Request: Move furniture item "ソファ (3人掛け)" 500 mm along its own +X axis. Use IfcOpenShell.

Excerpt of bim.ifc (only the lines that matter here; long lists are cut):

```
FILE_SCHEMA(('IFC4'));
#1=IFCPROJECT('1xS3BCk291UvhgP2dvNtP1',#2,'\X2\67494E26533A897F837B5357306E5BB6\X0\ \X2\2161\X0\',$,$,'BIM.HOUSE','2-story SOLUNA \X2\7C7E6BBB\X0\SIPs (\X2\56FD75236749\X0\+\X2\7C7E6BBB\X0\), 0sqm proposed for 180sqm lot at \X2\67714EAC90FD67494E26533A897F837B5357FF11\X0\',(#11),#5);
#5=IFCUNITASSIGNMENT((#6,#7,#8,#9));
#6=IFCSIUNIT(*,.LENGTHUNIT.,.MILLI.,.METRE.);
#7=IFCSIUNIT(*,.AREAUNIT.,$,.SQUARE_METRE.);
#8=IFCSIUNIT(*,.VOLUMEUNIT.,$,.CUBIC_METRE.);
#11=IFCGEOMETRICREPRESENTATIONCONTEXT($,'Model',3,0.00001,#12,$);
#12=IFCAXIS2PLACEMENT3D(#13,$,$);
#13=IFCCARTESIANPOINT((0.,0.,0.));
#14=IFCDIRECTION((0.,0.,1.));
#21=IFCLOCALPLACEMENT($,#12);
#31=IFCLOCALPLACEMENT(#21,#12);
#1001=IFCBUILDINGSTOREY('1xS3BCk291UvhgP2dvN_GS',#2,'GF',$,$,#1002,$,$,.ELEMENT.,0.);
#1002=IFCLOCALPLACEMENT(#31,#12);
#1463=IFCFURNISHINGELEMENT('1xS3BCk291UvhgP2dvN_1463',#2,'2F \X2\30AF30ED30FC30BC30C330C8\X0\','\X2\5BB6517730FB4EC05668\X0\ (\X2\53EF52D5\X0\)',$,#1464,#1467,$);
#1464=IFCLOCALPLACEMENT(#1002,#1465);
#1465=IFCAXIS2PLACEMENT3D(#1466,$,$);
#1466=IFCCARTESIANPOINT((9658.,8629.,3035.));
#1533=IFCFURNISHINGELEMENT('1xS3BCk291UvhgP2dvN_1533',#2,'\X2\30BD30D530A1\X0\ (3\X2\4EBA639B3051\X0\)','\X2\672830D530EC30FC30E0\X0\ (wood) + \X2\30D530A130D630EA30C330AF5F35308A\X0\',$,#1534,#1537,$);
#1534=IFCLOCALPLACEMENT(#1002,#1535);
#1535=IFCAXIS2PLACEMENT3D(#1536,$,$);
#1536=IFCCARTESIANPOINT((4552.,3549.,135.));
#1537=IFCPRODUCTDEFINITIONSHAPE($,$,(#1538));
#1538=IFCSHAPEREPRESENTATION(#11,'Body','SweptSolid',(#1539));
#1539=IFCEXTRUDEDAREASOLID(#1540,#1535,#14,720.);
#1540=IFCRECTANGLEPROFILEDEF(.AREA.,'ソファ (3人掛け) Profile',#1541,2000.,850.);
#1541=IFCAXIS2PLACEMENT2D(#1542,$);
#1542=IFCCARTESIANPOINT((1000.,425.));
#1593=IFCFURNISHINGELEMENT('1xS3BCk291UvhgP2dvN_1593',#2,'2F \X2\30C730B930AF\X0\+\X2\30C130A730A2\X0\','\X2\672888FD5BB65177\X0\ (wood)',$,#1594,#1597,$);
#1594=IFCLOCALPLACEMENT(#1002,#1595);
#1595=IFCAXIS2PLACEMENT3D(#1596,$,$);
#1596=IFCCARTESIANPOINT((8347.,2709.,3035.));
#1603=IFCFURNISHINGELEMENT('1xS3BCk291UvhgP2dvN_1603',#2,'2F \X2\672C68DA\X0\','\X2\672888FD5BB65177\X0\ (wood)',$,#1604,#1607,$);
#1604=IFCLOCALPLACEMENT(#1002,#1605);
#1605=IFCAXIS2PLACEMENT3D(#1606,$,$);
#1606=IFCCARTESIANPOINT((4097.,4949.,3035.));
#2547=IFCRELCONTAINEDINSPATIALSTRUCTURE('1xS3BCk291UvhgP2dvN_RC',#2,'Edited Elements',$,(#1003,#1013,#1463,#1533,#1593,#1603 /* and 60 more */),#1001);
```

```python
import ifcopenshell
import ifcopenshell.api.geometry
import ifcopenshell.util.placement

model = ifcopenshell.open("bim.ifc")

item = model.by_id(1533)
matrix = ifcopenshell.util.placement.get_local_placement(item.ObjectPlacement)
matrix[:3, 3] += matrix[:3, 0] * 500.0
ifcopenshell.api.geometry.edit_object_placement(model, product=item, matrix=matrix, is_si=False)

print(ifcopenshell.util.placement.get_local_placement(item.ObjectPlacement).round(3) + 0.0)

model.write("bim_rev.ifc")
```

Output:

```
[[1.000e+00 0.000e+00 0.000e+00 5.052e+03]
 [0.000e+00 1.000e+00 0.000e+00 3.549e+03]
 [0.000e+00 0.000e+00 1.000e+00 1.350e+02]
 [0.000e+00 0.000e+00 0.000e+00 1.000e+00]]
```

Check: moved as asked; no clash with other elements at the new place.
